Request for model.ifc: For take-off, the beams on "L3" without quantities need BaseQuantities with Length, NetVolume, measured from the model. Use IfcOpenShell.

First a look at what the model holds.

```python
import ifcopenshell
import ifcopenshell.util.element
import ifcopenshell.util.unit

model = ifcopenshell.open("model.ifc")
print(model.schema)
for unit_type in ("LENGTHUNIT", "AREAUNIT", "VOLUMEUNIT"):
    print(unit_type, ifcopenshell.util.unit.calculate_unit_scale(model, unit_type))
storey = next(s for s in model.by_type("IfcBuildingStorey") if s.Name == "L3")
beams = [e for e in ifcopenshell.util.element.get_decomposition(storey) if e.is_a("IfcBeam")]
for e in sorted(beams, key=lambda e: e.id()):
    print(e.id(), e.is_a(), e.Name, list(ifcopenshell.util.element.get_psets(e, qtos_only=True)), sep=" | ")
```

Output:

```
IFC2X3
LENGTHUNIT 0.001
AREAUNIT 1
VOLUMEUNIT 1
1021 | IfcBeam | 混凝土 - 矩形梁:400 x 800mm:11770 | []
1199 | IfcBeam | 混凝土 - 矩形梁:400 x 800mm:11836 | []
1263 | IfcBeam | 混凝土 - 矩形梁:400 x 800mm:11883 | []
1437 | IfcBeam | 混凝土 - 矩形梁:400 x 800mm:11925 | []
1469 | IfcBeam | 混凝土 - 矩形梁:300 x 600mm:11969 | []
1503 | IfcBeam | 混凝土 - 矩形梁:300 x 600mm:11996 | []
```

```python
import ifcopenshell
import ifcopenshell.api.pset
import ifcopenshell.geom
import ifcopenshell.util.element
import ifcopenshell.util.shape
import ifcopenshell.util.unit

model = ifcopenshell.open("model.ifc")
unit_scale = ifcopenshell.util.unit.calculate_unit_scale(model)
volume_scale = ifcopenshell.util.unit.calculate_unit_scale(model, "VOLUMEUNIT")
settings = ifcopenshell.geom.settings()

storey = next(s for s in model.by_type("IfcBuildingStorey") if s.Name == "L3")
beams = [e for e in ifcopenshell.util.element.get_decomposition(storey) if e.is_a("IfcBeam")]

for e in sorted(beams, key=lambda e: e.id()):
    if ifcopenshell.util.element.get_psets(e, qtos_only=True, should_inherit=False):
        continue
    # Geometry comes back in metres, in the element's own axes.
    shape = ifcopenshell.geom.create_shape(settings, e)
    values = {
        "Length": ifcopenshell.util.shape.get_max_xyz(shape.geometry) / unit_scale,
        "NetVolume": ifcopenshell.util.shape.get_volume(shape.geometry) / volume_scale,
    }
    qto = ifcopenshell.api.pset.add_qto(model, product=e, name="BaseQuantities")
    ifcopenshell.api.pset.edit_qto(model, qto=qto, properties=values)
    print(e.id(), {k: round(v, 3) for k, v in values.items()})

model.write("model_v2.ifc")
```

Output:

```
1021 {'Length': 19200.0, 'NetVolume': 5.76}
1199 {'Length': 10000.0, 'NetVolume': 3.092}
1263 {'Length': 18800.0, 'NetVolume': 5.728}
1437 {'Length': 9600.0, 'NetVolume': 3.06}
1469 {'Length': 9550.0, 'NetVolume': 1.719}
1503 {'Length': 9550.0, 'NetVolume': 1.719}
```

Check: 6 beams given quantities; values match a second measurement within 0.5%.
